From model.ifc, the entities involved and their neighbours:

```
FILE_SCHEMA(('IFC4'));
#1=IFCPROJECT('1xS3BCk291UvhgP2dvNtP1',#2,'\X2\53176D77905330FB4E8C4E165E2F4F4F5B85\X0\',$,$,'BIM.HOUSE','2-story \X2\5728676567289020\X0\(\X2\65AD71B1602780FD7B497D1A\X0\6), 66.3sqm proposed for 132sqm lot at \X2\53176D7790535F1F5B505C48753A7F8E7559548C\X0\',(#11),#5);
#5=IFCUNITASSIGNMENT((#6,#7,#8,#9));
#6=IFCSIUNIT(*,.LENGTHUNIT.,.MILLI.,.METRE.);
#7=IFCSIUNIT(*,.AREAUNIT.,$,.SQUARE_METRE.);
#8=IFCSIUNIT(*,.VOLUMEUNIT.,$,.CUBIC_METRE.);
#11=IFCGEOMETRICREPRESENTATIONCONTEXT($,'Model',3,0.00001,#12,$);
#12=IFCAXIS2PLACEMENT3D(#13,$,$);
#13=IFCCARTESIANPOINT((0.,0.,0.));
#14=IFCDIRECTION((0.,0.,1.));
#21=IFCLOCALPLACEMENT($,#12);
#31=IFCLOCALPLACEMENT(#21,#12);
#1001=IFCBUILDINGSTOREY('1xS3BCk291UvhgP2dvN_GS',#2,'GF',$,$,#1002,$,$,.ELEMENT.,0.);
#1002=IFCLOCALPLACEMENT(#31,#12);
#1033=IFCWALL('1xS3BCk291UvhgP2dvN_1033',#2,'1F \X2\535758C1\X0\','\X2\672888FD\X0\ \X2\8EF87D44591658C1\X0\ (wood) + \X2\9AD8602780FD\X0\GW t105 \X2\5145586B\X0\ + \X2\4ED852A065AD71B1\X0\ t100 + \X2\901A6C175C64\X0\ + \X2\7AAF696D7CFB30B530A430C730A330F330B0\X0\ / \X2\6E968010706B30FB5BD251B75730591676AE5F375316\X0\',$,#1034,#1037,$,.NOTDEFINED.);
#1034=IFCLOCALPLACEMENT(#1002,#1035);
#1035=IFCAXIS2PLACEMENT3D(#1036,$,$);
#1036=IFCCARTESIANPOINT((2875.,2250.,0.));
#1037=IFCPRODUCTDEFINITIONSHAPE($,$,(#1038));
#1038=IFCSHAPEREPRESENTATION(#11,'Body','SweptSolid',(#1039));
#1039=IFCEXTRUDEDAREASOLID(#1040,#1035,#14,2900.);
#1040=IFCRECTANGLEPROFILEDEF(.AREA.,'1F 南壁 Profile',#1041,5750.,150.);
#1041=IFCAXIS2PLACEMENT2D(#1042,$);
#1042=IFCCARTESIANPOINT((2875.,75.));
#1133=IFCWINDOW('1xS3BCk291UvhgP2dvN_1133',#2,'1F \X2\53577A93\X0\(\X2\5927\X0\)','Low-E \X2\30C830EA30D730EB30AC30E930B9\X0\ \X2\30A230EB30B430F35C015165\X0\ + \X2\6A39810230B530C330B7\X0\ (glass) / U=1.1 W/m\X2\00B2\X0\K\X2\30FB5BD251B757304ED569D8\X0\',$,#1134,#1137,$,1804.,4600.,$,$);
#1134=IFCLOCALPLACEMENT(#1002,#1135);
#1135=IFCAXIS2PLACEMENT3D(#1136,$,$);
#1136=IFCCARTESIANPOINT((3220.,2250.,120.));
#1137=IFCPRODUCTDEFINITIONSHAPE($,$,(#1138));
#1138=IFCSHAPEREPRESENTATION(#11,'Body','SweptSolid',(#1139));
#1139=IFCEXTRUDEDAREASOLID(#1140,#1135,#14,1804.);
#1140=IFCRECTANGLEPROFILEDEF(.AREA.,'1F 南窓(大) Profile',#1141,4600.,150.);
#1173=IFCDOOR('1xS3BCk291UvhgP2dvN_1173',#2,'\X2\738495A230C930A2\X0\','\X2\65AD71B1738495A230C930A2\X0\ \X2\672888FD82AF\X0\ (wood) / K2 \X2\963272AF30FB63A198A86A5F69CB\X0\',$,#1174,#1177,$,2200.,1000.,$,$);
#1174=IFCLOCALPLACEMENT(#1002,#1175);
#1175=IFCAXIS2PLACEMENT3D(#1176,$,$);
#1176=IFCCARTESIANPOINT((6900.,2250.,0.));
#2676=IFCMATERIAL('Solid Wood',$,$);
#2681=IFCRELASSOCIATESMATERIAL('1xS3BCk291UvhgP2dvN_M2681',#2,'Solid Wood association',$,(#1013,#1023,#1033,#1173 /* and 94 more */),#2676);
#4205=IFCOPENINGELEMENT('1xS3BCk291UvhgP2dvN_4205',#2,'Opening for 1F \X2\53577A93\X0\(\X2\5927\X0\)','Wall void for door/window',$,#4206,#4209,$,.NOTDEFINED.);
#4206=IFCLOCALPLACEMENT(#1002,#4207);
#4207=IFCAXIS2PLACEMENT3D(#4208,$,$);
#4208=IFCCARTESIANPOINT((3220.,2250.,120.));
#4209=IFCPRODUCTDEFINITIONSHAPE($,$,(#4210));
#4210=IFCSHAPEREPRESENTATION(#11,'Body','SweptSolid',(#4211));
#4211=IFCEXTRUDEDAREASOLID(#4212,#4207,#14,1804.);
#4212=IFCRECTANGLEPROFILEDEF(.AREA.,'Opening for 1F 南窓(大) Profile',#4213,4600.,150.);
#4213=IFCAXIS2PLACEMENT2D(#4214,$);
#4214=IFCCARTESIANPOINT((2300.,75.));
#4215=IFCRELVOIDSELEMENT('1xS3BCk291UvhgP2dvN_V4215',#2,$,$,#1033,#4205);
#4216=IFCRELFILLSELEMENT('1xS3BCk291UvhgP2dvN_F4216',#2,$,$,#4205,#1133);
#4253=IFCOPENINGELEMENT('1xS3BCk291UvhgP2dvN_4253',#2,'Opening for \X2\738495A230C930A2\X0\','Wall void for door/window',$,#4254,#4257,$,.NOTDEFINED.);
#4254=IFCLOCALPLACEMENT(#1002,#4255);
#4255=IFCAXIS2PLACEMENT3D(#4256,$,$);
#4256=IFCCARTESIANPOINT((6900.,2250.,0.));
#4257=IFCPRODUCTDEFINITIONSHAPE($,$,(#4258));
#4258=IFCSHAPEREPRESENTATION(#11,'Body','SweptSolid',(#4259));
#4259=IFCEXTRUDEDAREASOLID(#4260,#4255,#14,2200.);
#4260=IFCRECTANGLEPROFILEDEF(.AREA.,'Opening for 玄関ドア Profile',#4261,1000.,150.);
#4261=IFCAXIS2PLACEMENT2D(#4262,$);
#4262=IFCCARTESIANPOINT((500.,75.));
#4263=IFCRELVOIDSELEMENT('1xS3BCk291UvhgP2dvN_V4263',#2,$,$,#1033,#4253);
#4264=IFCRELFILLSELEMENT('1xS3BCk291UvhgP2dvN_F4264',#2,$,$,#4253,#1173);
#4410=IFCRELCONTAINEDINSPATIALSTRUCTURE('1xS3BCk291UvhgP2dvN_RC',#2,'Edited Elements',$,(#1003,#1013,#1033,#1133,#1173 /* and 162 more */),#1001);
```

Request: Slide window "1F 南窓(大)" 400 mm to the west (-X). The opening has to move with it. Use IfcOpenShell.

```python
import ifcopenshell
import ifcopenshell.api.geometry
import ifcopenshell.util.placement
import ifcopenshell.util.unit

model = ifcopenshell.open("model.ifc")
unit_scale = ifcopenshell.util.unit.calculate_unit_scale(model)

window = model.by_guid("1xS3BCk291UvhgP2dvN_1133")
opening = window.FillsVoids[0].RelatingOpeningElement
wall = opening.VoidsElements[0].RelatingBuildingElement

wall_matrix = ifcopenshell.util.placement.get_local_placement(wall.ObjectPlacement)
shift = wall_matrix[:3, 0] * -0.4 / unit_scale
before = ifcopenshell.util.placement.get_local_placement(window.ObjectPlacement)[:3, 3].copy()

# The window is not placed relative to its opening, so move both.
for product in (opening, window):
    matrix = ifcopenshell.util.placement.get_local_placement(product.ObjectPlacement)
    matrix[:3, 3] += shift
    ifcopenshell.api.geometry.edit_object_placement(model, product=product, matrix=matrix, is_si=False)

after = ifcopenshell.util.placement.get_local_placement(window.ObjectPlacement)[:3, 3]
print("window moved by", (after - before).round(3) + 0.0)

model.write("model-out.ifc")
```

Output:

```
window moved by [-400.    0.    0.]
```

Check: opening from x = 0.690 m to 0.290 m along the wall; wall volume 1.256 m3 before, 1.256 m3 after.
